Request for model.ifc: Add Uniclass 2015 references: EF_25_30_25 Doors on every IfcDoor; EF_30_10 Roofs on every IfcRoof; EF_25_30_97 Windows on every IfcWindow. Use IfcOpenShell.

First a look at what the model holds.

```python
import ifcopenshell

model = ifcopenshell.open("model.ifc")
print(model.schema)
print("classifications:", [c.Name for c in model.by_type("IfcClassification")])
for ifc_class in ("IfcDoor", "IfcRoof", "IfcStair", "IfcWall", "IfcWindow"):
    print(ifc_class, len(model.by_type(ifc_class)))
```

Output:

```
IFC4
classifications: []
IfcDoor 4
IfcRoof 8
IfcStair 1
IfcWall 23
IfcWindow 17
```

```python
import ifcopenshell
import ifcopenshell.api.classification

model = ifcopenshell.open("model.ifc")

system = ifcopenshell.api.classification.add_classification(model, classification="Uniclass 2015")

codes = {
    "IfcDoor": ("EF_25_30_25", "Doors"),
    "IfcRoof": ("EF_30_10", "Roofs"),
    "IfcWindow": ("EF_25_30_97", "Windows"),
}
for ifc_class, (code, name) in codes.items():
    products = model.by_type(ifc_class)
    ifcopenshell.api.classification.add_reference(
        model, products=products, classification=system, identification=code, name=name
    )
    print(code, len(products))

model.write("model_v2.ifc")
```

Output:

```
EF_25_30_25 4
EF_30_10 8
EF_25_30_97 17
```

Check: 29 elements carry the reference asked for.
